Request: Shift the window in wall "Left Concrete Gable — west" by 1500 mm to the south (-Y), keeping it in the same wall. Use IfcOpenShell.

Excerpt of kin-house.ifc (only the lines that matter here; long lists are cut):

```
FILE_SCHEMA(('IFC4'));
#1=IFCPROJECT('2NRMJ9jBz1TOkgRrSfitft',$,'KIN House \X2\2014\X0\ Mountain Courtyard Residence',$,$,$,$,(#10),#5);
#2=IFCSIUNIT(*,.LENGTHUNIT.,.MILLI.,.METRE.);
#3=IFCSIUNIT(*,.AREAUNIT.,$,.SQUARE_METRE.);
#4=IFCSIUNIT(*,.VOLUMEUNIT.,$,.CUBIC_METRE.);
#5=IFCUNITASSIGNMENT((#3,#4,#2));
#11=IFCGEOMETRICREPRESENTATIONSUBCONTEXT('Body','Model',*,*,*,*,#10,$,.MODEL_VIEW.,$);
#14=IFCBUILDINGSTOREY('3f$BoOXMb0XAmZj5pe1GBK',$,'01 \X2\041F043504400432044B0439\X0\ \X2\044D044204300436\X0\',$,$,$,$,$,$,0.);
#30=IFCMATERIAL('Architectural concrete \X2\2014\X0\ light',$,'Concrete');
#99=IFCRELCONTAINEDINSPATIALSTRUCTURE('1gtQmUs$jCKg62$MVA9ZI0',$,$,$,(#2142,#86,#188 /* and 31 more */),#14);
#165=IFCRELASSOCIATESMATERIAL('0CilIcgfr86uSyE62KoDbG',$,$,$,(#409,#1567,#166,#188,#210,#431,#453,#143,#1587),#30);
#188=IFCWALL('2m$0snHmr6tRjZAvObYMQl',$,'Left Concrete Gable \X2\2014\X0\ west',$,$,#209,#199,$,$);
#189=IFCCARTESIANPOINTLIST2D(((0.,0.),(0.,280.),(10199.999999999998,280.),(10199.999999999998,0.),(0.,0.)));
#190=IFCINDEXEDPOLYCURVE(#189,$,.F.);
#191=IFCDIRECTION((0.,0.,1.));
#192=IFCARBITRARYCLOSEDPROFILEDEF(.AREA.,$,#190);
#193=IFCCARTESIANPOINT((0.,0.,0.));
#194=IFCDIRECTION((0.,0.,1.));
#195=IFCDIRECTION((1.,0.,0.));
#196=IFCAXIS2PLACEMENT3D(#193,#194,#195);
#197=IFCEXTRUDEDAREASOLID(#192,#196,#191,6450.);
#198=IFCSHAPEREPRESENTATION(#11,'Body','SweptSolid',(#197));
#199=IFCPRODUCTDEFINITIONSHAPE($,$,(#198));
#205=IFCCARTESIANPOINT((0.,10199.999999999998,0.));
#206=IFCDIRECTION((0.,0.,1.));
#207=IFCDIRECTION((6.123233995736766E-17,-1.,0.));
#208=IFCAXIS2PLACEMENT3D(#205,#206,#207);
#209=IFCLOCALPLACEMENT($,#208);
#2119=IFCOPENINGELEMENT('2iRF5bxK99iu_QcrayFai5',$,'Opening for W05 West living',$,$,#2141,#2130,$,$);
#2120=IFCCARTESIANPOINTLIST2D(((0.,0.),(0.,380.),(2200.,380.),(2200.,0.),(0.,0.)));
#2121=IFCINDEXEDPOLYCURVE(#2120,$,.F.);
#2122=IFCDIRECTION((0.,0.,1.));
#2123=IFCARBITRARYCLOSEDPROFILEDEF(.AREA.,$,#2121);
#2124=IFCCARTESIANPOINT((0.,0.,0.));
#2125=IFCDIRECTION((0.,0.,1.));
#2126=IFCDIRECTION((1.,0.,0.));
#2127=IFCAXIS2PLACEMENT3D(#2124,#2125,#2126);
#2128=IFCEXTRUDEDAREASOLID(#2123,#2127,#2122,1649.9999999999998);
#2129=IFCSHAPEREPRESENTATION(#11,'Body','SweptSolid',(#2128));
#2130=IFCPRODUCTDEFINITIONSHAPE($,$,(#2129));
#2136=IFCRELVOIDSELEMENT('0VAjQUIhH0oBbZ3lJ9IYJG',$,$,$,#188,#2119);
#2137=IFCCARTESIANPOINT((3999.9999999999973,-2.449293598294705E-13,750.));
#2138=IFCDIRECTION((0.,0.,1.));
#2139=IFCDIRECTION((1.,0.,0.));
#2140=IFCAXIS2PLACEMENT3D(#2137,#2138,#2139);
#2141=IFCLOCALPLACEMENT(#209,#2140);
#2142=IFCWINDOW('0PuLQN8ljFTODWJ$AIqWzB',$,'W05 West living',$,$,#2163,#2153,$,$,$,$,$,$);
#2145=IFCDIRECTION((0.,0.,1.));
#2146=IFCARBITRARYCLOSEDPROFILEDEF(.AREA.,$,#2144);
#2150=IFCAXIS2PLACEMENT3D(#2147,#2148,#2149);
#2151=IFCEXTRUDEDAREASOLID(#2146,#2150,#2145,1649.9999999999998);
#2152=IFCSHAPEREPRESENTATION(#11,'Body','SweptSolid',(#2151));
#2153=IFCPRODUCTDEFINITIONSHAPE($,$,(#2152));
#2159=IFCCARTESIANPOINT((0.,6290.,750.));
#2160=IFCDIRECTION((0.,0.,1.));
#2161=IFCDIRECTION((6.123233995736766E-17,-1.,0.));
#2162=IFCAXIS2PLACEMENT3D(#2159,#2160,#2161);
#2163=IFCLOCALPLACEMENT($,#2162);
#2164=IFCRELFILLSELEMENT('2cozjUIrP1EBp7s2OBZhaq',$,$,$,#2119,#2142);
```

```python
import ifcopenshell
import ifcopenshell.api.geometry
import ifcopenshell.util.placement
import ifcopenshell.util.unit

model = ifcopenshell.open("kin-house.ifc")
unit_scale = ifcopenshell.util.unit.calculate_unit_scale(model)

window = model.by_guid("0PuLQN8ljFTODWJ$AIqWzB")
opening = window.FillsVoids[0].RelatingOpeningElement
wall = opening.VoidsElements[0].RelatingBuildingElement

wall_matrix = ifcopenshell.util.placement.get_local_placement(wall.ObjectPlacement)
shift = wall_matrix[:3, 0] * 1.5 / unit_scale
before = ifcopenshell.util.placement.get_local_placement(window.ObjectPlacement)[:3, 3].copy()

# The window is not placed relative to its opening, so move both.
for product in (opening, window):
    matrix = ifcopenshell.util.placement.get_local_placement(product.ObjectPlacement)
    matrix[:3, 3] += shift
    ifcopenshell.api.geometry.edit_object_placement(model, product=product, matrix=matrix, is_si=False)

after = ifcopenshell.util.placement.get_local_placement(window.ObjectPlacement)[:3, 3]
print("window moved by", (after - before).round(3) + 0.0)

model.write("kin-house_edited.ifc")
```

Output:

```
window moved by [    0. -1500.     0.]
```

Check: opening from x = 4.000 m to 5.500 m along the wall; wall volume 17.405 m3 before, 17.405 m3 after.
